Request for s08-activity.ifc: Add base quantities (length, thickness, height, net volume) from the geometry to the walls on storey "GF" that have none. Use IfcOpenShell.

First a look at what the model holds.

```python
import ifcopenshell
import ifcopenshell.util.element
import ifcopenshell.util.unit

model = ifcopenshell.open("s08-activity.ifc")
print(model.schema)
for unit_type in ("LENGTHUNIT", "AREAUNIT", "VOLUMEUNIT"):
    print(unit_type, ifcopenshell.util.unit.calculate_unit_scale(model, unit_type))
storey = next(s for s in model.by_type("IfcBuildingStorey") if s.Name == "GF")
walls = [e for e in ifcopenshell.util.element.get_decomposition(storey) if e.is_a("IfcWall")]
for e in sorted(walls, key=lambda e: e.id()):
    print(e.id(), e.is_a(), e.Name, list(ifcopenshell.util.element.get_psets(e, qtos_only=True)), sep=" | ")
```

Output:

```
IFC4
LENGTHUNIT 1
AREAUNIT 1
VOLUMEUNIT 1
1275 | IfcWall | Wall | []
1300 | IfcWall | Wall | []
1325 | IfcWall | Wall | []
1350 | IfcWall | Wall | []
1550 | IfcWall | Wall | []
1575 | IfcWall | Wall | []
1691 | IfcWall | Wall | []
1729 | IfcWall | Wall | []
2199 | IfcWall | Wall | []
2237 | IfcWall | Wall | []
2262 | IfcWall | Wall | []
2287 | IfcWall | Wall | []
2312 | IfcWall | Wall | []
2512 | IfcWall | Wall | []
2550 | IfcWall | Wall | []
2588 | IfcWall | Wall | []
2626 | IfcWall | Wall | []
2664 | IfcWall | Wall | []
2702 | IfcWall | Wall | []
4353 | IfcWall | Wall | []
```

```python
import ifcopenshell
import ifcopenshell.api.pset
import ifcopenshell.geom
import ifcopenshell.util.element
import ifcopenshell.util.shape
import ifcopenshell.util.unit

model = ifcopenshell.open("s08-activity.ifc")
unit_scale = ifcopenshell.util.unit.calculate_unit_scale(model)
volume_scale = ifcopenshell.util.unit.calculate_unit_scale(model, "VOLUMEUNIT")
settings = ifcopenshell.geom.settings()

storey = next(s for s in model.by_type("IfcBuildingStorey") if s.Name == "GF")
walls = [e for e in ifcopenshell.util.element.get_decomposition(storey) if e.is_a("IfcWall")]

for e in sorted(walls, key=lambda e: e.id()):
    if ifcopenshell.util.element.get_psets(e, qtos_only=True, should_inherit=False):
        continue
    # Geometry comes back in metres, in the element's own axes.
    shape = ifcopenshell.geom.create_shape(settings, e)
    values = {
        "Length": ifcopenshell.util.shape.get_x(shape.geometry) / unit_scale,
        "Width": ifcopenshell.util.shape.get_y(shape.geometry) / unit_scale,
        "Height": ifcopenshell.util.shape.get_z(shape.geometry) / unit_scale,
        "NetVolume": ifcopenshell.util.shape.get_volume(shape.geometry) / volume_scale,
    }
    qto = ifcopenshell.api.pset.add_qto(model, product=e, name="Qto_WallBaseQuantities")
    ifcopenshell.api.pset.edit_qto(model, qto=qto, properties=values)
    print(e.id(), {k: round(v, 3) for k, v in values.items()})

model.write("s08-activity_rev.ifc")
```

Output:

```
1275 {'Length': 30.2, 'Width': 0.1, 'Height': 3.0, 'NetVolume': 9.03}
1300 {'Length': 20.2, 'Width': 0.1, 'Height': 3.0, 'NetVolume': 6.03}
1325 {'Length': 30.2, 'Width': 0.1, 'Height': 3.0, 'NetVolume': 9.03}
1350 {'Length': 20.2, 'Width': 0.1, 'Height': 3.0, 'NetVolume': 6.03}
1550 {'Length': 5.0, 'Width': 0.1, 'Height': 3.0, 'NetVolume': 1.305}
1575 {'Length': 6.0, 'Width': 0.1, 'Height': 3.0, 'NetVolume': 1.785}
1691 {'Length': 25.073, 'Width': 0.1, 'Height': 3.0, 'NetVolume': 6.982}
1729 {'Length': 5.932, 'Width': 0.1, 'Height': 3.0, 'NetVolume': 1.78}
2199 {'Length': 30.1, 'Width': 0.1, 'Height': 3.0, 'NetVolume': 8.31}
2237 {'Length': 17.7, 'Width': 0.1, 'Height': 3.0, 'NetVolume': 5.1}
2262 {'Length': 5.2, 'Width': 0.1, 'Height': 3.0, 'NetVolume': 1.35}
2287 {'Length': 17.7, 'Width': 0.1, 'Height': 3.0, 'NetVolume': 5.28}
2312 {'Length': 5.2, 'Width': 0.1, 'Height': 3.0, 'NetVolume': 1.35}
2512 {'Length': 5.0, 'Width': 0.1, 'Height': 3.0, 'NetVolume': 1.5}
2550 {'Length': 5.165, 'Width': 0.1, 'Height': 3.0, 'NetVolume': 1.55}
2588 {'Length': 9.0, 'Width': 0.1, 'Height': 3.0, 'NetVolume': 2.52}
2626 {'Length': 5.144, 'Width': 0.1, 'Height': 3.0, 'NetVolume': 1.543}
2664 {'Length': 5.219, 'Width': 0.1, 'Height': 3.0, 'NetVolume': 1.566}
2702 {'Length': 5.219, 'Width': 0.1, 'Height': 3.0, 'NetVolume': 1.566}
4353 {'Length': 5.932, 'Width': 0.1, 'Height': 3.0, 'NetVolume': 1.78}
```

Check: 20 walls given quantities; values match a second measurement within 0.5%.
